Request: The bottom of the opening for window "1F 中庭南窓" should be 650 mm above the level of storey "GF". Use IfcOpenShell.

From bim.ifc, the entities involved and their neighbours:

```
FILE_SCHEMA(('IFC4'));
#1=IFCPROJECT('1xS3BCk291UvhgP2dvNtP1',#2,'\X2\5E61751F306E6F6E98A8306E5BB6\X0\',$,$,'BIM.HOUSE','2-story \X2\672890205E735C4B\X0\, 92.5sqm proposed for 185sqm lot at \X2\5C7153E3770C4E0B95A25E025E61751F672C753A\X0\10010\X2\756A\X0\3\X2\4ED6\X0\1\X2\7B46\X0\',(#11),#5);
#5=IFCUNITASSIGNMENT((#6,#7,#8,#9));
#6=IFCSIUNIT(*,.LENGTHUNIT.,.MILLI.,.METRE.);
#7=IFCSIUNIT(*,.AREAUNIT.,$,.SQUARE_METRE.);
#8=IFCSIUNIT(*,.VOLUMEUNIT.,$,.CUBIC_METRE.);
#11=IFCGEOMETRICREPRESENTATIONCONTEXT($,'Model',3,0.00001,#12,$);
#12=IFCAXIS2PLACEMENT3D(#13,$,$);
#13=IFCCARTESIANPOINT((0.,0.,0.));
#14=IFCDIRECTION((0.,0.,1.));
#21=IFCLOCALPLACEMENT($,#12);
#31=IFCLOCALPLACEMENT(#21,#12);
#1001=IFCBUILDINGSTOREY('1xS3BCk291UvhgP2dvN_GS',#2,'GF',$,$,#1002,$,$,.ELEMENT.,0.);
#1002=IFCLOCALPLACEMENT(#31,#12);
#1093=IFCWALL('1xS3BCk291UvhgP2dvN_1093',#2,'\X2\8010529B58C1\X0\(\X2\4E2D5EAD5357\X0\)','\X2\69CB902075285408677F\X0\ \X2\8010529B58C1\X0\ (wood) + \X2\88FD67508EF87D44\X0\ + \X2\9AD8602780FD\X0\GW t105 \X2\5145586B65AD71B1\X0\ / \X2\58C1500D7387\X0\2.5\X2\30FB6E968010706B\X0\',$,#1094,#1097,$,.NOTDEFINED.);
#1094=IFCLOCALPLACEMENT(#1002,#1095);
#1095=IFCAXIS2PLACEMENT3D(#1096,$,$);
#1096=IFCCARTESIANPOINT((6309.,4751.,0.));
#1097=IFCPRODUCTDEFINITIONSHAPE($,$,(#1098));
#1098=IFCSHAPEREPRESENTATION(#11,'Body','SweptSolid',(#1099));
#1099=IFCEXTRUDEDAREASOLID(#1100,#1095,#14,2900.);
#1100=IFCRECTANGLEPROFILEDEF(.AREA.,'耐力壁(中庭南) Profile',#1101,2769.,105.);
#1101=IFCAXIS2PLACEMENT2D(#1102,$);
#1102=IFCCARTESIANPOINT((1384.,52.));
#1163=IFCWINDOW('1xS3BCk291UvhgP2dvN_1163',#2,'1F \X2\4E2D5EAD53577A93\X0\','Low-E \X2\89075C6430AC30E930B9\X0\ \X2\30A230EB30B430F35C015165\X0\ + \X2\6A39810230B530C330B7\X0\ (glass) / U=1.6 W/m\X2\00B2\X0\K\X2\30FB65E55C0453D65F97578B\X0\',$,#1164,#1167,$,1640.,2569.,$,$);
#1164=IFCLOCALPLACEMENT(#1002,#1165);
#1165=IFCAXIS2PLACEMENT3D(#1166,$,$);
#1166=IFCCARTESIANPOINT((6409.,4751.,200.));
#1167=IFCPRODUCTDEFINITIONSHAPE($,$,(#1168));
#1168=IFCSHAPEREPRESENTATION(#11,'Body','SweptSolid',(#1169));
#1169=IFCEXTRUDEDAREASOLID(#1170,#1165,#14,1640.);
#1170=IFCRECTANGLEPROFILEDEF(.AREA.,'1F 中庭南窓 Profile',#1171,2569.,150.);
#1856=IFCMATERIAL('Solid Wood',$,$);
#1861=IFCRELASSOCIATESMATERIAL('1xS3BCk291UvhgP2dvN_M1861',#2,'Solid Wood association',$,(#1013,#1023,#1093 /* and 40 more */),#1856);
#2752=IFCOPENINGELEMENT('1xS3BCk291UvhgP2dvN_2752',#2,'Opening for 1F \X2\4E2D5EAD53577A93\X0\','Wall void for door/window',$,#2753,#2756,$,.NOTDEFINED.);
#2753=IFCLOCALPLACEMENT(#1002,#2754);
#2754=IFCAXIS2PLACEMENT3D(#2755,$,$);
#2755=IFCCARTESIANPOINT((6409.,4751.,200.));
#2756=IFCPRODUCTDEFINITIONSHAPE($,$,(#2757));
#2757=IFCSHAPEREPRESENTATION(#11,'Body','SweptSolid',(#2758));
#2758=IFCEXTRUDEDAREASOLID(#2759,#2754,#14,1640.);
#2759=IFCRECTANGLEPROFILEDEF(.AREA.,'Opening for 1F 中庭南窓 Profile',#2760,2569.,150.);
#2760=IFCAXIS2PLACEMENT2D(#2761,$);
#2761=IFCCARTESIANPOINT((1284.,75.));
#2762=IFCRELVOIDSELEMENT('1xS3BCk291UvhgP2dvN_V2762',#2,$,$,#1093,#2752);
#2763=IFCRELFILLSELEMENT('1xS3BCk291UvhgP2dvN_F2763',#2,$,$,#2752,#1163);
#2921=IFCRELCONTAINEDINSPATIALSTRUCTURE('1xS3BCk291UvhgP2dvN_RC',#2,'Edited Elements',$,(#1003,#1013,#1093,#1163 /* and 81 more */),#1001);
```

```python
import numpy as np
import ifcopenshell
import ifcopenshell.api.geometry
import ifcopenshell.geom
import ifcopenshell.util.element
import ifcopenshell.util.placement
import ifcopenshell.util.shape
import ifcopenshell.util.unit

model = ifcopenshell.open("bim.ifc")
unit_scale = ifcopenshell.util.unit.calculate_unit_scale(model)

window = model.by_guid("1xS3BCk291UvhgP2dvN_1163")
opening = window.FillsVoids[0].RelatingOpeningElement
storey = ifcopenshell.util.element.get_container(window, ifc_class="IfcBuildingStorey")
level = ifcopenshell.util.placement.get_local_placement(storey.ObjectPlacement)[2, 3]

# The opening's origin need not be at the sill, so measure its lowest point.
shape = ifcopenshell.geom.create_shape(ifcopenshell.geom.settings(), opening)
bottom = ifcopenshell.util.shape.get_shape_bottom_elevation(shape, shape.geometry) / unit_scale
dz = level + 0.65 / unit_scale - bottom

shift = np.array([0.0, 0.0, dz])
# The window is not placed relative to its opening, so move both.
for product in (opening, window):
    matrix = ifcopenshell.util.placement.get_local_placement(product.ObjectPlacement)
    matrix[:3, 3] += shift
    ifcopenshell.api.geometry.edit_object_placement(model, product=product, matrix=matrix, is_si=False)

print(f"moved by {dz * unit_scale:+.3f} m")

model.write("bim_rev.ifc")
```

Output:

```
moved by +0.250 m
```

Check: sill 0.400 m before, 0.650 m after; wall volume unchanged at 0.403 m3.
